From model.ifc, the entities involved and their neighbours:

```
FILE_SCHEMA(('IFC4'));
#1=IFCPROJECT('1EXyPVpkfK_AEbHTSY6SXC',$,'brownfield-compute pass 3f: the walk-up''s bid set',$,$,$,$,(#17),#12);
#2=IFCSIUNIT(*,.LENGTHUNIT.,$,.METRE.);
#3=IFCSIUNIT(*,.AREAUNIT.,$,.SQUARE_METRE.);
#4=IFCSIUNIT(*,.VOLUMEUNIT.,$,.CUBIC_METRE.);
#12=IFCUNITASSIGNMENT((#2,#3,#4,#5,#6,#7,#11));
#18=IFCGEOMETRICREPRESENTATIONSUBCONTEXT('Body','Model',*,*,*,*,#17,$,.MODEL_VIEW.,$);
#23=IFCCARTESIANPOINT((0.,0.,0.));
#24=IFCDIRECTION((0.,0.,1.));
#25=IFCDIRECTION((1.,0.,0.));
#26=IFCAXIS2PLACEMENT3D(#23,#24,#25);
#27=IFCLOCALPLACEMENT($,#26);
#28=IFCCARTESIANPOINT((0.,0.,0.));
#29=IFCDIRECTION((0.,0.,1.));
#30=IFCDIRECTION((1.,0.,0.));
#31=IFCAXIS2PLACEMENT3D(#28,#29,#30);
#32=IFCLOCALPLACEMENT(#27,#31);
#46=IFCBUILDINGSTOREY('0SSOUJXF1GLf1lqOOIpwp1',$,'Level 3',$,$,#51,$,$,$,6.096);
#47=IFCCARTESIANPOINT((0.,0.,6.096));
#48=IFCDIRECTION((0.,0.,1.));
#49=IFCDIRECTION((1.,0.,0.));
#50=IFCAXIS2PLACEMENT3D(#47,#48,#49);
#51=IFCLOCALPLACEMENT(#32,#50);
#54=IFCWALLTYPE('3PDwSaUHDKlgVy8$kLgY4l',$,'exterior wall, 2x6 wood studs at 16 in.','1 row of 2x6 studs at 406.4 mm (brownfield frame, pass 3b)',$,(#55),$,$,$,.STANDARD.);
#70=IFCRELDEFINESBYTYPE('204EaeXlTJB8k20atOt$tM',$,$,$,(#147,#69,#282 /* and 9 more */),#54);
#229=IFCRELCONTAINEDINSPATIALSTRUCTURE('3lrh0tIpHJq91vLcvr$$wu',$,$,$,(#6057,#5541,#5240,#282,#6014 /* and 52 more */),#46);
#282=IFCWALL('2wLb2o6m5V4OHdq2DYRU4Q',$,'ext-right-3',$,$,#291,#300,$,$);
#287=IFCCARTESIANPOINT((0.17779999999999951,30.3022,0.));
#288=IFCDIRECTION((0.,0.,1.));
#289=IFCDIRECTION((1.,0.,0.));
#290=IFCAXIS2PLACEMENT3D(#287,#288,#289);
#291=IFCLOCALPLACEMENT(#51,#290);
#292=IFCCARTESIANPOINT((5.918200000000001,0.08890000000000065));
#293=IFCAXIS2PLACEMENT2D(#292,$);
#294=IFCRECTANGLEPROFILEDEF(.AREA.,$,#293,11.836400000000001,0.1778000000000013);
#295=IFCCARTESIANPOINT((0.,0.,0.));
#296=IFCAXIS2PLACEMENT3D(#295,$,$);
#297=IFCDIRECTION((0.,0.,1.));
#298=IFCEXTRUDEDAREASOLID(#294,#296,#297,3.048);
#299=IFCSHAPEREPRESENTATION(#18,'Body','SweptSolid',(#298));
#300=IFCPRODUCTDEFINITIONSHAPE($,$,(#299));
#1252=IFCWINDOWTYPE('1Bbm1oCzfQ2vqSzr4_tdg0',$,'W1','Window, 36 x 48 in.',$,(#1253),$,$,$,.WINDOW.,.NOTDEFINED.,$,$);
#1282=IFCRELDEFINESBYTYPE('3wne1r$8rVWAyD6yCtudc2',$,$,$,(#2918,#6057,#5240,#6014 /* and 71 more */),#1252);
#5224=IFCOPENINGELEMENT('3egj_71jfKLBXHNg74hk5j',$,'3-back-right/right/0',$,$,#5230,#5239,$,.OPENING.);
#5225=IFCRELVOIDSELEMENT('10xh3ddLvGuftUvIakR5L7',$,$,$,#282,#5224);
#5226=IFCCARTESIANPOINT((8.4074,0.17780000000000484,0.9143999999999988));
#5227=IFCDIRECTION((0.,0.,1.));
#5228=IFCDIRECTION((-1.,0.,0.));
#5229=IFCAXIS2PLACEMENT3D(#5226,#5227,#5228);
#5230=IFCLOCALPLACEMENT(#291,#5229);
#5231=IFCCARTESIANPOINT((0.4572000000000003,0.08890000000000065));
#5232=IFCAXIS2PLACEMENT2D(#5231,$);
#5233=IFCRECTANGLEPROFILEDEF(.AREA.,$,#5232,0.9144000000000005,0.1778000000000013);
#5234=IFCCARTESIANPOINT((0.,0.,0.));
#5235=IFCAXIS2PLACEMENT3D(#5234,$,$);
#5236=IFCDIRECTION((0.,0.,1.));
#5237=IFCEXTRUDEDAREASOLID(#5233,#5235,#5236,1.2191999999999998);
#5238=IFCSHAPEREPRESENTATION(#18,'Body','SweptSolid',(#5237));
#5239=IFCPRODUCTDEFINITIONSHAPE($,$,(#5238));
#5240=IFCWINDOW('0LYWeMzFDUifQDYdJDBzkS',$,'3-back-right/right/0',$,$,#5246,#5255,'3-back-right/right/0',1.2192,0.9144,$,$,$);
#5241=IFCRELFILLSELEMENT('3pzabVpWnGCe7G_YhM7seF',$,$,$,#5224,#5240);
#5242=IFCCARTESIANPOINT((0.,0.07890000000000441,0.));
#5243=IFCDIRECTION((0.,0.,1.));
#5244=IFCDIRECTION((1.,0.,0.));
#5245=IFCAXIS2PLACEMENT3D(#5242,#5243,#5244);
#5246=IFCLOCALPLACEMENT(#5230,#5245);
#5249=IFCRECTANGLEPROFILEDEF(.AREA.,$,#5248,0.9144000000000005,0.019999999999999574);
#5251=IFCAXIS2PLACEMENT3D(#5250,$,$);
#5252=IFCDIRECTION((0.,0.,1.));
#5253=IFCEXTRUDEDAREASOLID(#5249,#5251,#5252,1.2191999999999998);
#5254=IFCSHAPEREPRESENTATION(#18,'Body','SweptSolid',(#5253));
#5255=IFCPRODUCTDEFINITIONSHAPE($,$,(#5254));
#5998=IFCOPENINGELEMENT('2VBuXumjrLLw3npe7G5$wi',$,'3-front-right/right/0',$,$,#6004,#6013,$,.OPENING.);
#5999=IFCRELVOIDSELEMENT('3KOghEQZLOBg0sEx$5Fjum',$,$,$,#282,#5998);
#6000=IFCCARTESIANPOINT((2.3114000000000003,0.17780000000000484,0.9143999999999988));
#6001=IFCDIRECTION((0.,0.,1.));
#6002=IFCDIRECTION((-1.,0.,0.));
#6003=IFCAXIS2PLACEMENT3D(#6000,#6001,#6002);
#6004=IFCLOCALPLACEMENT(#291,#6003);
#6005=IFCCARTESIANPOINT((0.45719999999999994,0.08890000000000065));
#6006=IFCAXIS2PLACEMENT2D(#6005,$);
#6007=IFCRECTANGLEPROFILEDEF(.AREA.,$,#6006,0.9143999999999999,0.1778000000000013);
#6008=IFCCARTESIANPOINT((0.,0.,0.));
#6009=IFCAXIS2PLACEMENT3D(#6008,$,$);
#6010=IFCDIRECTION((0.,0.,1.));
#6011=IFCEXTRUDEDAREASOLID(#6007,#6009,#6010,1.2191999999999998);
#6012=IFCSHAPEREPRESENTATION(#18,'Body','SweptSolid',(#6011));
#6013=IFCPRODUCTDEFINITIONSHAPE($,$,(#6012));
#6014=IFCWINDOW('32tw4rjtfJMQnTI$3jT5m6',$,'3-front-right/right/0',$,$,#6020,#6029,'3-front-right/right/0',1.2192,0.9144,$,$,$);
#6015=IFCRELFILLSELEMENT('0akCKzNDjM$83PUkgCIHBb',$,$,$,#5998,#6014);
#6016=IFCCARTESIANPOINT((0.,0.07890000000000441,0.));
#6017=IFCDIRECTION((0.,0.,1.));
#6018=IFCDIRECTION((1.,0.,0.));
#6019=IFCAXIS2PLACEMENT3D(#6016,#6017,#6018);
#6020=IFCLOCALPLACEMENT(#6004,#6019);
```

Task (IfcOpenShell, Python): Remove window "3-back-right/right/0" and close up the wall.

```python
import ifcopenshell
import ifcopenshell.api.feature
import ifcopenshell.api.root
import ifcopenshell.geom
import ifcopenshell.util.shape

model = ifcopenshell.open("model.ifc")
settings = ifcopenshell.geom.settings()


def volume(element):
    """Net volume in cubic metres, openings subtracted."""
    shape = ifcopenshell.geom.create_shape(settings, element)
    return ifcopenshell.util.shape.get_volume(shape.geometry)


window = model.by_guid("0LYWeMzFDUifQDYdJDBzkS")
opening = window.FillsVoids[0].RelatingOpeningElement
wall = opening.VoidsElements[0].RelatingBuildingElement
before = volume(wall)

ifcopenshell.api.root.remove_product(model, product=window)
ifcopenshell.api.feature.remove_feature(model, feature=opening)

after = volume(wall)

print(f"wall volume {before:.3f} -> {after:.3f} m3")

model.write("model-out.ifc")
```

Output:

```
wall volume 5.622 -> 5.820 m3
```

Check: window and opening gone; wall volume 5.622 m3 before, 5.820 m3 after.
